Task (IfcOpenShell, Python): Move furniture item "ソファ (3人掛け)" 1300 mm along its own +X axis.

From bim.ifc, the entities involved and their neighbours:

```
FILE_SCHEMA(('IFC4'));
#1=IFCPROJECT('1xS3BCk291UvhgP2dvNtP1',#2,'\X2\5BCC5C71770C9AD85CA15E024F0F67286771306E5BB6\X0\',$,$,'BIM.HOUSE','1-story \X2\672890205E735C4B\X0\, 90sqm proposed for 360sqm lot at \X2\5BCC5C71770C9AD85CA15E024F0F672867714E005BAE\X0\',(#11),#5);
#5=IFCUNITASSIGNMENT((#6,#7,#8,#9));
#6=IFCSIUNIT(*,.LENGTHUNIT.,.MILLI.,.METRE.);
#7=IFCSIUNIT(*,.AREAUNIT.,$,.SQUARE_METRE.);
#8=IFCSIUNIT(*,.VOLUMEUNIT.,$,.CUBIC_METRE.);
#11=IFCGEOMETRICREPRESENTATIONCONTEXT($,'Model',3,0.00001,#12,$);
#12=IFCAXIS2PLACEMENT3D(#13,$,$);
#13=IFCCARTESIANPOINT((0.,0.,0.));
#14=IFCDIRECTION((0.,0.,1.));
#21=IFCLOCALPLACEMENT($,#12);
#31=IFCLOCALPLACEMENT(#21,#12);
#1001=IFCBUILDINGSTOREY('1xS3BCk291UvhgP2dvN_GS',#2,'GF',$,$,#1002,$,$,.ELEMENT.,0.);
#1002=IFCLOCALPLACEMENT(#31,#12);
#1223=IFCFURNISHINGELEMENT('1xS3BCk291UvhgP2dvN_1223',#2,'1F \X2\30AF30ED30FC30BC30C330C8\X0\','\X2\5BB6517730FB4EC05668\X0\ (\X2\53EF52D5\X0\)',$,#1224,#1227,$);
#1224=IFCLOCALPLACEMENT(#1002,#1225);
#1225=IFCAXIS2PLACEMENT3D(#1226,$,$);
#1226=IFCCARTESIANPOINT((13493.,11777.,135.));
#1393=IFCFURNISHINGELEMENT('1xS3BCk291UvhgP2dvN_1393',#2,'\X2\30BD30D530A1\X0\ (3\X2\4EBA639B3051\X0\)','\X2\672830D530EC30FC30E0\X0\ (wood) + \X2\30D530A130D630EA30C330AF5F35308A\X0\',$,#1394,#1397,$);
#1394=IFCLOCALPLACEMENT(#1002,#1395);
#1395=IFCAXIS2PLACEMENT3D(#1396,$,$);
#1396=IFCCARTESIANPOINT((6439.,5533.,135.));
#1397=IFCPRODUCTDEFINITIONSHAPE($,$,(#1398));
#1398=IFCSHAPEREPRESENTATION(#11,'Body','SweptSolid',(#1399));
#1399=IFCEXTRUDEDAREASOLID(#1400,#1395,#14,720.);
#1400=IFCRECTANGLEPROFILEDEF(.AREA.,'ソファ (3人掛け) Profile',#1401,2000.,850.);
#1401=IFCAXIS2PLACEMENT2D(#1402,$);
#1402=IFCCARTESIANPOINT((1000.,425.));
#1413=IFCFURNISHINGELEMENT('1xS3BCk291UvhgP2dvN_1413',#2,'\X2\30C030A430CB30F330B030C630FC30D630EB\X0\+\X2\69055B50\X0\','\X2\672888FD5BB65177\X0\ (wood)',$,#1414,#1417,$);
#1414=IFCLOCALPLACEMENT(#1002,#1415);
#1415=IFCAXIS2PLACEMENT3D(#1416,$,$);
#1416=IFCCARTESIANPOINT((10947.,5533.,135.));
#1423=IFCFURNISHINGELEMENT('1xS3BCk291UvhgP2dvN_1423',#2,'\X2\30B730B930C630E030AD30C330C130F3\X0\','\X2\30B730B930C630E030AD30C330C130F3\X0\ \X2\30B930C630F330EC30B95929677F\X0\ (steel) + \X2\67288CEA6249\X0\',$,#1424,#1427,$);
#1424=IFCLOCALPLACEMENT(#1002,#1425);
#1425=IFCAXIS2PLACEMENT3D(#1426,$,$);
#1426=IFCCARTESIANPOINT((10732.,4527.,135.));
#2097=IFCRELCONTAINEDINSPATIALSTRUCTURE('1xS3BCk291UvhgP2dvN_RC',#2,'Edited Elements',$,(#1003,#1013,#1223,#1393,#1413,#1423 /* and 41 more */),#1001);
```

```python
import ifcopenshell
import ifcopenshell.api.geometry
import ifcopenshell.util.placement
import ifcopenshell.util.unit

model = ifcopenshell.open("bim.ifc")
unit_scale = ifcopenshell.util.unit.calculate_unit_scale(model)

item = model.by_guid("1xS3BCk291UvhgP2dvN_1393")
matrix = ifcopenshell.util.placement.get_local_placement(item.ObjectPlacement)
matrix[:3, 3] += matrix[:3, 0] * 1.3 / unit_scale
ifcopenshell.api.geometry.edit_object_placement(model, product=item, matrix=matrix, is_si=False)

print(ifcopenshell.util.placement.get_local_placement(item.ObjectPlacement).round(3) + 0.0)

model.write("bim-out.ifc")
```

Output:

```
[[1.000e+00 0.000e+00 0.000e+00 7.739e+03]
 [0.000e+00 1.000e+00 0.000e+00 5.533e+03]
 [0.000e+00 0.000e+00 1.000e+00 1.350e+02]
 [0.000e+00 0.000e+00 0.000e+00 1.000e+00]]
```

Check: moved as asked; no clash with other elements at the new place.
